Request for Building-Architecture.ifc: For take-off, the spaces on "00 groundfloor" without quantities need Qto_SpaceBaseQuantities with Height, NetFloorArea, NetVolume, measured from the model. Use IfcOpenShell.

First a look at what the model holds.

```python
import ifcopenshell
import ifcopenshell.util.element
import ifcopenshell.util.unit

model = ifcopenshell.open("Building-Architecture.ifc")
print(model.schema)
for unit_type in ("LENGTHUNIT", "AREAUNIT", "VOLUMEUNIT"):
    print(unit_type, ifcopenshell.util.unit.calculate_unit_scale(model, unit_type))
storey = next(s for s in model.by_type("IfcBuildingStorey") if s.Name == "00 groundfloor")
spaces = [e for e in ifcopenshell.util.element.get_decomposition(storey) if e.is_a("IfcSpace")]
for e in sorted(spaces, key=lambda e: e.id()):
    print(e.id(), e.is_a(), e.Name, list(ifcopenshell.util.element.get_psets(e, qtos_only=True)), sep=" | ")
```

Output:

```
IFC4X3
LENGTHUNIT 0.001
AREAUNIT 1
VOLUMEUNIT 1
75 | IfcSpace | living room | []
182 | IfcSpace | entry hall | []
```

```python
import ifcopenshell
import ifcopenshell.api.pset
import ifcopenshell.geom
import ifcopenshell.util.element
import ifcopenshell.util.shape
import ifcopenshell.util.unit

model = ifcopenshell.open("Building-Architecture.ifc")
unit_scale = ifcopenshell.util.unit.calculate_unit_scale(model)
area_scale = ifcopenshell.util.unit.calculate_unit_scale(model, "AREAUNIT")
volume_scale = ifcopenshell.util.unit.calculate_unit_scale(model, "VOLUMEUNIT")
settings = ifcopenshell.geom.settings()

storey = next(s for s in model.by_type("IfcBuildingStorey") if s.Name == "00 groundfloor")
spaces = [e for e in ifcopenshell.util.element.get_decomposition(storey) if e.is_a("IfcSpace")]

for e in sorted(spaces, key=lambda e: e.id()):
    if ifcopenshell.util.element.get_psets(e, qtos_only=True, should_inherit=False):
        continue
    # Geometry comes back in metres, in the element's own axes.
    shape = ifcopenshell.geom.create_shape(settings, e)
    values = {
        "Height": ifcopenshell.util.shape.get_z(shape.geometry) / unit_scale,
        "NetFloorArea": ifcopenshell.util.shape.get_footprint_area(shape.geometry) / area_scale,
        "NetVolume": ifcopenshell.util.shape.get_volume(shape.geometry) / volume_scale,
    }
    qto = ifcopenshell.api.pset.add_qto(model, product=e, name="Qto_SpaceBaseQuantities")
    ifcopenshell.api.pset.edit_qto(model, qto=qto, properties=values)
    print(e.id(), {k: round(v, 3) for k, v in values.items()})

model.write("Building-Architecture_v2.ifc")
```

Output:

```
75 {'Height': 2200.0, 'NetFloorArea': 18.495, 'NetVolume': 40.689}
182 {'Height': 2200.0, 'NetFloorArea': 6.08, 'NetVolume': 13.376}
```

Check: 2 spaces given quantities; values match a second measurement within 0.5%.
